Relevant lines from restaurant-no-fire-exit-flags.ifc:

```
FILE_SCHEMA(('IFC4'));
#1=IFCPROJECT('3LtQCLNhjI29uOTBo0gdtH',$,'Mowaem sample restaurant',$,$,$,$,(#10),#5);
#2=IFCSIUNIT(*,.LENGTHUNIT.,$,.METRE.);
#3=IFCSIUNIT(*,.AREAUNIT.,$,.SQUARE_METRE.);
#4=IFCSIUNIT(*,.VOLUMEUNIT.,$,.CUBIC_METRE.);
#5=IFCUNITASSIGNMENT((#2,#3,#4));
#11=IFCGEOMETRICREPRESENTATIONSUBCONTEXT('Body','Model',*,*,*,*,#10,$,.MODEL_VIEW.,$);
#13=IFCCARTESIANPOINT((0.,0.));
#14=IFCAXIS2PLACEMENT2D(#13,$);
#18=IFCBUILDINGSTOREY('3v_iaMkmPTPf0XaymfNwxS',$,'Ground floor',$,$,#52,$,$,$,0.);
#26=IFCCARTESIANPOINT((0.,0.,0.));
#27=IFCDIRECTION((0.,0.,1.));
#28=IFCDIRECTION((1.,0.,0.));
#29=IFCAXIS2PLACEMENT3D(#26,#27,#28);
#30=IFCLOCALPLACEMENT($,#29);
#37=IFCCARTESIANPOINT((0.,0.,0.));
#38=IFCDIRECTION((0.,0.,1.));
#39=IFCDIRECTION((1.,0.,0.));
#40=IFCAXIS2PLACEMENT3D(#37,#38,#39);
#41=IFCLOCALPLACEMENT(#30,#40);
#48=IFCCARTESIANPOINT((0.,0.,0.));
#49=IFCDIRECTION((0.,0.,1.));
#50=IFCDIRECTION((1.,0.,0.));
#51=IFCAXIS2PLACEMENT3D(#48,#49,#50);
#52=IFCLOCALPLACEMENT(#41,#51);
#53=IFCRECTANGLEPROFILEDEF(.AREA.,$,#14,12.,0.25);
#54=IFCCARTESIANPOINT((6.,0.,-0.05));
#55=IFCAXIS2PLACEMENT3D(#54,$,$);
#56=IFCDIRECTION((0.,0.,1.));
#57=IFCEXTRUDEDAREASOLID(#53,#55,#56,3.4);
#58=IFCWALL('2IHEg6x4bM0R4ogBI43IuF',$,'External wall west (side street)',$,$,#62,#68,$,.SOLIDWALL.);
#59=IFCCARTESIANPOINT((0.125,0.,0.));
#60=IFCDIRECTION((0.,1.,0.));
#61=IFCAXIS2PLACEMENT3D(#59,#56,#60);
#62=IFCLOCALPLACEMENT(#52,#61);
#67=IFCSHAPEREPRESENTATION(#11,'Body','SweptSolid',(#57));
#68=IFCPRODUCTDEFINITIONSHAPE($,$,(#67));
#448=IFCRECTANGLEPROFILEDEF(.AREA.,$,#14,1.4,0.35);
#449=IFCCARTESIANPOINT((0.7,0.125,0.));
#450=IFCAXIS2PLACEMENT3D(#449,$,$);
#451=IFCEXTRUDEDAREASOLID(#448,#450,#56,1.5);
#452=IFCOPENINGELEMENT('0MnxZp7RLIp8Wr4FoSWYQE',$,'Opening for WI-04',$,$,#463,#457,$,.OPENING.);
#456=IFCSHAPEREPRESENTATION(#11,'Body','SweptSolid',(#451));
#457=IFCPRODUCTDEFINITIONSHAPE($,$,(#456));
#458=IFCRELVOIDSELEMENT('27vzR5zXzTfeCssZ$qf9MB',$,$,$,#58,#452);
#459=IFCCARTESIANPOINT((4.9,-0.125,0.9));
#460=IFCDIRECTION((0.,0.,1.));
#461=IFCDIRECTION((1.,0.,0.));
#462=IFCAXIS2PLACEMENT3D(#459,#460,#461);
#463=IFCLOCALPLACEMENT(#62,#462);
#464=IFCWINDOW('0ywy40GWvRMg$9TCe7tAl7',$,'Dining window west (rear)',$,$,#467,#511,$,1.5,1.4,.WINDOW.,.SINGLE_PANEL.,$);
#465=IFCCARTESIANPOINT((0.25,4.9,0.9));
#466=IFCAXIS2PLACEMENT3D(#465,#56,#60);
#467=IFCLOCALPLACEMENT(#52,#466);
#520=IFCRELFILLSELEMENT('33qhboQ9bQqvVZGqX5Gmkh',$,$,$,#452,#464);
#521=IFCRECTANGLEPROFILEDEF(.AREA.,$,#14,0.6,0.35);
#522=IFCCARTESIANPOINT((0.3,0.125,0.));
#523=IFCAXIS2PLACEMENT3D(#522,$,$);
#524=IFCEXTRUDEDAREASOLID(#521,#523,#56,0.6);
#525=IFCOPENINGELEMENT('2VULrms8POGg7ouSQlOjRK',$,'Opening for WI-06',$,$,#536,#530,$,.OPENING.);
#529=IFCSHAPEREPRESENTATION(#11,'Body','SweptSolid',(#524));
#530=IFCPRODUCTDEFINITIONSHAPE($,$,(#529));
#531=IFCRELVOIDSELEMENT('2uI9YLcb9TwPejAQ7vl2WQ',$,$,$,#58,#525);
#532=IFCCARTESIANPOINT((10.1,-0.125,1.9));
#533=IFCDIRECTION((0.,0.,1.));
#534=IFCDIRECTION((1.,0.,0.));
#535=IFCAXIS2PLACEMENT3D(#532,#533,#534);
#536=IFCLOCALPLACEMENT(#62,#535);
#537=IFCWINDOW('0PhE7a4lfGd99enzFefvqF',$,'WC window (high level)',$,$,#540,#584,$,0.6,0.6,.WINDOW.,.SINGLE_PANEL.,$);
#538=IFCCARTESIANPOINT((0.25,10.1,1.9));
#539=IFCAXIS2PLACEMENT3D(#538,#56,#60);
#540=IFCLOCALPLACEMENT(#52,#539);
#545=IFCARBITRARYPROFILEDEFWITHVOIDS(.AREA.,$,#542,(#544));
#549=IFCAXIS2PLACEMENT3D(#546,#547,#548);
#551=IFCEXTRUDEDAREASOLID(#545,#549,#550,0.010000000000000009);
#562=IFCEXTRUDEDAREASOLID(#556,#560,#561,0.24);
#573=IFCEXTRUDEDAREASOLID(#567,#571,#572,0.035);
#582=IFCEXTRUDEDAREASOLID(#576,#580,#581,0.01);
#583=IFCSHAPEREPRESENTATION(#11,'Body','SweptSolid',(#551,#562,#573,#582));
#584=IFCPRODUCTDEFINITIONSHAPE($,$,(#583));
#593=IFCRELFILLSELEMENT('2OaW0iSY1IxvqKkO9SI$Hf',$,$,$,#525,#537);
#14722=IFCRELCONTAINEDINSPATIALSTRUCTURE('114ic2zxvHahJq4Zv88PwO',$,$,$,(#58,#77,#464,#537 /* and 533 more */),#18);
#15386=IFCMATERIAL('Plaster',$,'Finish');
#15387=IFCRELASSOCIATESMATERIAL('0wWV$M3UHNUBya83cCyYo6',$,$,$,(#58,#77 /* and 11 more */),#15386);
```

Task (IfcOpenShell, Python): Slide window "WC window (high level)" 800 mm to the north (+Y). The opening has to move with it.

```python
import ifcopenshell
import ifcopenshell.api.geometry
import ifcopenshell.util.placement
import ifcopenshell.util.unit

model = ifcopenshell.open("restaurant-no-fire-exit-flags.ifc")
unit_scale = ifcopenshell.util.unit.calculate_unit_scale(model)

window = model.by_guid("0PhE7a4lfGd99enzFefvqF")
opening = window.FillsVoids[0].RelatingOpeningElement
wall = opening.VoidsElements[0].RelatingBuildingElement

wall_matrix = ifcopenshell.util.placement.get_local_placement(wall.ObjectPlacement)
shift = wall_matrix[:3, 0] * 0.8 / unit_scale
before = ifcopenshell.util.placement.get_local_placement(window.ObjectPlacement)[:3, 3].copy()

# The window is not placed relative to its opening, so move both.
for product in (opening, window):
    matrix = ifcopenshell.util.placement.get_local_placement(product.ObjectPlacement)
    matrix[:3, 3] += shift
    ifcopenshell.api.geometry.edit_object_placement(model, product=product, matrix=matrix, is_si=False)

after = ifcopenshell.util.placement.get_local_placement(window.ObjectPlacement)[:3, 3]
print("window moved by", (after - before).round(3) + 0.0)

model.write("restaurant-no-fire-exit-flags_v2.ifc")
```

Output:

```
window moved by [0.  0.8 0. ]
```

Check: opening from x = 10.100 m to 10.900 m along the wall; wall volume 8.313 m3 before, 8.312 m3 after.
